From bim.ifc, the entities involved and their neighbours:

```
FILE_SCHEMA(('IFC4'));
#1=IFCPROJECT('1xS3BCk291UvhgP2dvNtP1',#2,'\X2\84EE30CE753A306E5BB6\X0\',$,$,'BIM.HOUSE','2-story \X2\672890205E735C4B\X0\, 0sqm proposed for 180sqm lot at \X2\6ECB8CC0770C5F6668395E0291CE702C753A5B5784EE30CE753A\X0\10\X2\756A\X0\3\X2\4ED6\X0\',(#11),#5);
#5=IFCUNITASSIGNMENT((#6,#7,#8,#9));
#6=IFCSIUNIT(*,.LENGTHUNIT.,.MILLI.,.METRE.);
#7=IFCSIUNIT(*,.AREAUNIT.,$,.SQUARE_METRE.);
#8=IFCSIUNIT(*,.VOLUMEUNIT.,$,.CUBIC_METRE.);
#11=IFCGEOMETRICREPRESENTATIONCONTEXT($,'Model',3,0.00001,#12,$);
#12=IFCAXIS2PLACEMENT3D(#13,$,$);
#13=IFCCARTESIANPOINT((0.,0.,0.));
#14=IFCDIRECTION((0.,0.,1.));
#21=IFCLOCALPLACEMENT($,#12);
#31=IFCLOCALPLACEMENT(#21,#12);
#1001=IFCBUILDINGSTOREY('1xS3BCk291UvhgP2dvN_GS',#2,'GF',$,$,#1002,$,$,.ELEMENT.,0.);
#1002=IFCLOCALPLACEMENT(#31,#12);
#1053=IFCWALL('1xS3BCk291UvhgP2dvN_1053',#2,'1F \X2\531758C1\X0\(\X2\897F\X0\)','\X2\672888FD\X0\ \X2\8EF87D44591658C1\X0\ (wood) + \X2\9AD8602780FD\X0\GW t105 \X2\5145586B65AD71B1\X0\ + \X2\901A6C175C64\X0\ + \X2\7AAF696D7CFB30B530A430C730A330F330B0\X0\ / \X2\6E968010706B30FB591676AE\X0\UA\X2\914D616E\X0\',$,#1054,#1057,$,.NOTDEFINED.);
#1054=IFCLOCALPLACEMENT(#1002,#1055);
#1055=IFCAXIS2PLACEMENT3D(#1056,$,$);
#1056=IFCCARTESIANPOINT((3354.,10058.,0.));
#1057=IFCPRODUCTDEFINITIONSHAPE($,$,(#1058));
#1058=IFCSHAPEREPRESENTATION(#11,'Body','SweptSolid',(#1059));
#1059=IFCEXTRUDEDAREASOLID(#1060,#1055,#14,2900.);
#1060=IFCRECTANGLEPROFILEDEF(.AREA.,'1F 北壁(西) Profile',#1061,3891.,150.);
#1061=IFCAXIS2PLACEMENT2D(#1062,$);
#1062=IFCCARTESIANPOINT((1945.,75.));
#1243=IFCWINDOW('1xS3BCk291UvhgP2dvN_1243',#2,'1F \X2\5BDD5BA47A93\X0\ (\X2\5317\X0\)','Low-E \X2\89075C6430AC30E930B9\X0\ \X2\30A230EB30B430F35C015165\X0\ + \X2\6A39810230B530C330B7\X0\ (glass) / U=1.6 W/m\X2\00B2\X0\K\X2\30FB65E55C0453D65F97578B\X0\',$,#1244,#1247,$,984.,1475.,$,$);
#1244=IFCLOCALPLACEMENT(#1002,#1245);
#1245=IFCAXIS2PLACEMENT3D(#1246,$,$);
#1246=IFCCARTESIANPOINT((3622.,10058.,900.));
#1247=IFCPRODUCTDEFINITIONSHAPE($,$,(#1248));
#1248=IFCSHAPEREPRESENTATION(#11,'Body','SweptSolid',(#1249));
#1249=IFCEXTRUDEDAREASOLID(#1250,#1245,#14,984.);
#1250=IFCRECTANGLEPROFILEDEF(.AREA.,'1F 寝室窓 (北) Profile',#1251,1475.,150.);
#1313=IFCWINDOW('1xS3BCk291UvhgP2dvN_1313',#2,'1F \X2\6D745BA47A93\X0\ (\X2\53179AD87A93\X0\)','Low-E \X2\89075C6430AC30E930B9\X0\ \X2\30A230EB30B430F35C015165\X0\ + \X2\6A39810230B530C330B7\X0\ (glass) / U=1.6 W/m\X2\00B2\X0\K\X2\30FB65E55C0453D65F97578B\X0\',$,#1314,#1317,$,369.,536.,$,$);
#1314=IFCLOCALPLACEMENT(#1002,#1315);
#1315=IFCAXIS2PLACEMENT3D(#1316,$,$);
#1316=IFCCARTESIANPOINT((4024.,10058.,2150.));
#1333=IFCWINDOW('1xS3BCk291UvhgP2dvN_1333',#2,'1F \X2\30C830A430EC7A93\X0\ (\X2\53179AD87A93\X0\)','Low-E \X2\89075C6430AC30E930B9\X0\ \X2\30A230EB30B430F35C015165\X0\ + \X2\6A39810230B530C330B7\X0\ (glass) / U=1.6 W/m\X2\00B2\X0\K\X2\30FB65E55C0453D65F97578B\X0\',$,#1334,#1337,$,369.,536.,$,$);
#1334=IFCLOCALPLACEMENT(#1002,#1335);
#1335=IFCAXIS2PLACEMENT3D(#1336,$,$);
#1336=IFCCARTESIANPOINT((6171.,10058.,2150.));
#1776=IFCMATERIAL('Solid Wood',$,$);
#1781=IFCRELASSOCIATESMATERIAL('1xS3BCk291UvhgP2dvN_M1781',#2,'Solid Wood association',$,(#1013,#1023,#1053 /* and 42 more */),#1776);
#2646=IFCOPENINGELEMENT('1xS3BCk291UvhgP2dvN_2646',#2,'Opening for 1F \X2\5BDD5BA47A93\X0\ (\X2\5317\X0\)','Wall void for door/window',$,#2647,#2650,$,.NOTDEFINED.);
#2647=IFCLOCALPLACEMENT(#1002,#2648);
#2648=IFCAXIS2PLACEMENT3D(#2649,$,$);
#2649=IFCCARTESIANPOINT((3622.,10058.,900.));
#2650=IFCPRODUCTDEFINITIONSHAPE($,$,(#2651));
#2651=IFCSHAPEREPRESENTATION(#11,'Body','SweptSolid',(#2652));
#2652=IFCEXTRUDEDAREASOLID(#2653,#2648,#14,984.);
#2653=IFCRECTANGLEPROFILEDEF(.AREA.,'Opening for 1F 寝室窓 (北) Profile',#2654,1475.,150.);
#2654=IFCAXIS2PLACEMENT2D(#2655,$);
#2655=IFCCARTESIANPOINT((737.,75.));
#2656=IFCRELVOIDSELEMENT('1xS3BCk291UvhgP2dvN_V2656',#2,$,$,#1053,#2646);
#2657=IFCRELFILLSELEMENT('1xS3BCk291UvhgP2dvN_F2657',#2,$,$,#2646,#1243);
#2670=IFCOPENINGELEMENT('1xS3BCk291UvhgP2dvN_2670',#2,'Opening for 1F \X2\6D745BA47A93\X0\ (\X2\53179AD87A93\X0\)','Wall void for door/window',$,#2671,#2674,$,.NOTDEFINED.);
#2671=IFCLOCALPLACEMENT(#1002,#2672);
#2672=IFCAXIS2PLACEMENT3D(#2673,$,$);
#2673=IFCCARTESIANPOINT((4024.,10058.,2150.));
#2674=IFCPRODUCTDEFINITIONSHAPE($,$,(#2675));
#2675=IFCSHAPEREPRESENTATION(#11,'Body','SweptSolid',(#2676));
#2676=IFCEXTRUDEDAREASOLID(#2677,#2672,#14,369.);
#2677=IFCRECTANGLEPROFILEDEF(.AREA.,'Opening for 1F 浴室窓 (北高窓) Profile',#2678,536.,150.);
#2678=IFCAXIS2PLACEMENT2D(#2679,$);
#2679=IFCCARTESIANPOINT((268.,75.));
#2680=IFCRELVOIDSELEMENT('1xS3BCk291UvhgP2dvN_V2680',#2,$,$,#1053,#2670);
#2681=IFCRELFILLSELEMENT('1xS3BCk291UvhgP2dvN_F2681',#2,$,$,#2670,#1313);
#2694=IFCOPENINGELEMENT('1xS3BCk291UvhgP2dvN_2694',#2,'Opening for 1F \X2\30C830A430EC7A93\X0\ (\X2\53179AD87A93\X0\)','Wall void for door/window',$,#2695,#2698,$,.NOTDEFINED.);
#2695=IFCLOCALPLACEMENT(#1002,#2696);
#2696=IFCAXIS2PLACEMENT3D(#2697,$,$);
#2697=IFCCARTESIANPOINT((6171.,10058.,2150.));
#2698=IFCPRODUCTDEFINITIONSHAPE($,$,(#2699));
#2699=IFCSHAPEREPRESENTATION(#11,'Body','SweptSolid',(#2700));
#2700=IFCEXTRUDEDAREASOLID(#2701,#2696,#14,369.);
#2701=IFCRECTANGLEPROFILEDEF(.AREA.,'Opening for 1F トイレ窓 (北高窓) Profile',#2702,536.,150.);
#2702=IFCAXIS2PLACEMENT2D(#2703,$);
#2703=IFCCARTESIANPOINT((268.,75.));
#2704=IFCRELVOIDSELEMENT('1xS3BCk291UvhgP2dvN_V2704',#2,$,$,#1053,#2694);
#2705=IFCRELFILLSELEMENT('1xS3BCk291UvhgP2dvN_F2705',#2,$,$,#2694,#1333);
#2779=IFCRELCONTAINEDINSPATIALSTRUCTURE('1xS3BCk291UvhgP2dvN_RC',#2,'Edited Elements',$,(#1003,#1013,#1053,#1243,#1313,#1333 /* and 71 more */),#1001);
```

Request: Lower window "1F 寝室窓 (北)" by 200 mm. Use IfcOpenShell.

```python
import numpy as np
import ifcopenshell
import ifcopenshell.api.geometry
import ifcopenshell.util.placement
import ifcopenshell.util.unit

model = ifcopenshell.open("bim.ifc")
unit_scale = ifcopenshell.util.unit.calculate_unit_scale(model)

window = model.by_guid("1xS3BCk291UvhgP2dvN_1243")
opening = window.FillsVoids[0].RelatingOpeningElement
dz = -200.0

shift = np.array([0.0, 0.0, dz])
# The window is not placed relative to its opening, so move both.
for product in (opening, window):
    matrix = ifcopenshell.util.placement.get_local_placement(product.ObjectPlacement)
    matrix[:3, 3] += shift
    ifcopenshell.api.geometry.edit_object_placement(model, product=product, matrix=matrix, is_si=False)

print(f"moved by {dz * unit_scale:+.3f} m")

model.write("bim_updated.ifc")
```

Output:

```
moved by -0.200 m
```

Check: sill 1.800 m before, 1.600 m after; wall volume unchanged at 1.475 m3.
